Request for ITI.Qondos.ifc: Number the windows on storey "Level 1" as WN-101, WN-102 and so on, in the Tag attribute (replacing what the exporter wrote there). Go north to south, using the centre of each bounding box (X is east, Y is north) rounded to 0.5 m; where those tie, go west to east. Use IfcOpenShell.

First a look at what the model holds.

```python
import ifcopenshell
import ifcopenshell.util.element
import ifcopenshell.util.placement

model = ifcopenshell.open("ITI.Qondos.ifc")
print(model.schema)
storey = next(s for s in model.by_type("IfcBuildingStorey") if s.Name == "Level 1")
windows = [e for e in ifcopenshell.util.element.get_decomposition(storey) if e.is_a("IfcWindow")]
for e in sorted(windows, key=lambda e: e.id()):
    origin = ifcopenshell.util.placement.get_local_placement(e.ObjectPlacement)[:3, 3]
    print(e.id(), e.Tag, e.Name, origin.round(2) + 0.0, sep=" | ")
```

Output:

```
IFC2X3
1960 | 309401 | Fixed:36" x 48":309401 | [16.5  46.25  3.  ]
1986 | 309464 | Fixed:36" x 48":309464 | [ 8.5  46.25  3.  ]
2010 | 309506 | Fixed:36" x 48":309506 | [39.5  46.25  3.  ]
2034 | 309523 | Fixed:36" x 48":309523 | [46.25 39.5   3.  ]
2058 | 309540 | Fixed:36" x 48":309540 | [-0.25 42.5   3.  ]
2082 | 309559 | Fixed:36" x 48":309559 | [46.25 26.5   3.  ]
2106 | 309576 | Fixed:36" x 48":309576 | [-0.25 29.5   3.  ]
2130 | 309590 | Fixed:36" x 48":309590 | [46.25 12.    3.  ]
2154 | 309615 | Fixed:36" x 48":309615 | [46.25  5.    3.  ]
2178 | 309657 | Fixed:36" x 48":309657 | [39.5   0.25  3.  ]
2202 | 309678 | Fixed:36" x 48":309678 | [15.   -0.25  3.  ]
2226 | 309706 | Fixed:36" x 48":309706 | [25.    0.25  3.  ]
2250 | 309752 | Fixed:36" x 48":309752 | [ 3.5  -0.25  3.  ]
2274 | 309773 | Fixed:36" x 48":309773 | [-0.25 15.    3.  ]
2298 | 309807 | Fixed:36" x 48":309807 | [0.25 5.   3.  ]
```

```python
import ifcopenshell
import ifcopenshell.geom
import ifcopenshell.util.element
import ifcopenshell.util.shape

model = ifcopenshell.open("ITI.Qondos.ifc")
settings = ifcopenshell.geom.settings()
settings.set("use-world-coords", True)


def centre(element):
    shape = ifcopenshell.geom.create_shape(settings, element)
    return ifcopenshell.util.shape.get_bbox_centroid(shape.geometry)


storey = next(s for s in model.by_type("IfcBuildingStorey") if s.Name == "Level 1")
windows = [e for e in ifcopenshell.util.element.get_decomposition(storey) if e.is_a("IfcWindow")]

# Insertion points can sit at a corner or the storey origin, so sort by the geometry (in metres).
centres = {e: centre(e) for e in windows}
windows.sort(key=lambda e: (-round(centres[e][1] / 0.5), centres[e][0]))

for i, e in enumerate(windows, start=1):
    number = f"WN-1{i:02d}"
    e.Tag = number
    print(e.id(), number)

model.write("ITI.Qondos_edited.ifc")
```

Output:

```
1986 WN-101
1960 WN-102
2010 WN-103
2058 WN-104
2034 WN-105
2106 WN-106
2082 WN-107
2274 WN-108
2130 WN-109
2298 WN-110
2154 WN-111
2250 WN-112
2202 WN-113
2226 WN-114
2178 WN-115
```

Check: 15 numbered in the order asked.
